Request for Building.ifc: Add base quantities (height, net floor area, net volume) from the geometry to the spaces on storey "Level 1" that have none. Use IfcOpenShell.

First a look at what the model holds.

```python
import ifcopenshell
import ifcopenshell.util.element
import ifcopenshell.util.unit

model = ifcopenshell.open("Building.ifc")
print(model.schema)
for unit_type in ("LENGTHUNIT", "AREAUNIT", "VOLUMEUNIT"):
    print(unit_type, ifcopenshell.util.unit.calculate_unit_scale(model, unit_type))
storey = next(s for s in model.by_type("IfcBuildingStorey") if s.Name == "Level 1")
spaces = [e for e in ifcopenshell.util.element.get_decomposition(storey) if e.is_a("IfcSpace")]
for e in sorted(spaces, key=lambda e: e.id()):
    print(e.id(), e.is_a(), e.Name, list(ifcopenshell.util.element.get_psets(e, qtos_only=True)), sep=" | ")
```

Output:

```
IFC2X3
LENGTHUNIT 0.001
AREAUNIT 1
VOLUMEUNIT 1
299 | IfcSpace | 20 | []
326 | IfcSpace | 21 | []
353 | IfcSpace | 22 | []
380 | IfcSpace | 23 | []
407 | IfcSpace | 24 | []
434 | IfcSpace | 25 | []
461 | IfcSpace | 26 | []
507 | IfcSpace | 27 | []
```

```python
import ifcopenshell
import ifcopenshell.api.pset
import ifcopenshell.geom
import ifcopenshell.util.element
import ifcopenshell.util.shape
import ifcopenshell.util.unit

model = ifcopenshell.open("Building.ifc")
unit_scale = ifcopenshell.util.unit.calculate_unit_scale(model)
area_scale = ifcopenshell.util.unit.calculate_unit_scale(model, "AREAUNIT")
volume_scale = ifcopenshell.util.unit.calculate_unit_scale(model, "VOLUMEUNIT")
settings = ifcopenshell.geom.settings()

storey = next(s for s in model.by_type("IfcBuildingStorey") if s.Name == "Level 1")
spaces = [e for e in ifcopenshell.util.element.get_decomposition(storey) if e.is_a("IfcSpace")]

for e in sorted(spaces, key=lambda e: e.id()):
    if ifcopenshell.util.element.get_psets(e, qtos_only=True, should_inherit=False):
        continue
    # Geometry comes back in metres, in the element's own axes.
    shape = ifcopenshell.geom.create_shape(settings, e)
    values = {
        "Height": ifcopenshell.util.shape.get_z(shape.geometry) / unit_scale,
        "NetFloorArea": ifcopenshell.util.shape.get_footprint_area(shape.geometry) / area_scale,
        "NetVolume": ifcopenshell.util.shape.get_volume(shape.geometry) / volume_scale,
    }
    qto = ifcopenshell.api.pset.add_qto(model, product=e, name="BaseQuantities")
    ifcopenshell.api.pset.edit_qto(model, qto=qto, properties=values)
    print(e.id(), {k: round(v, 3) for k, v in values.items()})

model.write("Building_rev.ifc")
```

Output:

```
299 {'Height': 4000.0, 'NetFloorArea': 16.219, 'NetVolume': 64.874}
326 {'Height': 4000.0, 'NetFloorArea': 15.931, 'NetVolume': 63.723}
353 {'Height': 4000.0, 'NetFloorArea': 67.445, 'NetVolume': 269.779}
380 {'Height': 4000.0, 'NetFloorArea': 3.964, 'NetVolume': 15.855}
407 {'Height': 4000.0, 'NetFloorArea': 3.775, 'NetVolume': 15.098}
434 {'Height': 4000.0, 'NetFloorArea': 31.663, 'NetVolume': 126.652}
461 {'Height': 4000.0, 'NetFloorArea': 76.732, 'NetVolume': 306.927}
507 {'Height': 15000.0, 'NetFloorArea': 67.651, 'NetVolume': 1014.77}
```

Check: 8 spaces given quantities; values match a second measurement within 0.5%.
